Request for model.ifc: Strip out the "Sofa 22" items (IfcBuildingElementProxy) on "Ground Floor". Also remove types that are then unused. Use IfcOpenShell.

First a look at what the model holds.

```python
import ifcopenshell
import ifcopenshell.util.element

model = ifcopenshell.open("model.ifc")
print(model.schema)
storey = next(s for s in model.by_type("IfcBuildingStorey") if s.Name == "Ground Floor")
proxies = [e for e in ifcopenshell.util.element.get_decomposition(storey) if e.is_a("IfcBuildingElementProxy")]
seen = {}
for e in proxies:
    element_type = ifcopenshell.util.element.get_type(e)
    name = element_type.Name if element_type not in (None, e) else None
    seen[name] = seen.get(name, 0) + 1
for name, count in sorted(seen.items(), key=str):
    print(count, "x", name)
```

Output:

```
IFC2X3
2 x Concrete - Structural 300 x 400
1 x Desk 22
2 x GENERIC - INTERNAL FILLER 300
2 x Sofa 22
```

```python
import ifcopenshell
import ifcopenshell.api.root
import ifcopenshell.util.element

model = ifcopenshell.open("model.ifc")

storey = next(s for s in model.by_type("IfcBuildingStorey") if s.Name == "Ground Floor")
proxies = [e for e in ifcopenshell.util.element.get_decomposition(storey) if e.is_a("IfcBuildingElementProxy")]
targets = [e for e in proxies if (t := ifcopenshell.util.element.get_type(e)) not in (None, e) and t.Name == "Sofa 22"]
types = {ifcopenshell.util.element.get_type(e) for e in targets} - {None, *targets}

for e in targets:
    ifcopenshell.api.root.remove_product(model, product=e)
print(len(targets), "removed")

unused = [t for t in types if not ifcopenshell.util.element.get_types(t)]
for t in unused:
    ifcopenshell.api.root.remove_product(model, product=t)
print(len(unused), "unused types removed")

model.write("model_rev.ifc")
```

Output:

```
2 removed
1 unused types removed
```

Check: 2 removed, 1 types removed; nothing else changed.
